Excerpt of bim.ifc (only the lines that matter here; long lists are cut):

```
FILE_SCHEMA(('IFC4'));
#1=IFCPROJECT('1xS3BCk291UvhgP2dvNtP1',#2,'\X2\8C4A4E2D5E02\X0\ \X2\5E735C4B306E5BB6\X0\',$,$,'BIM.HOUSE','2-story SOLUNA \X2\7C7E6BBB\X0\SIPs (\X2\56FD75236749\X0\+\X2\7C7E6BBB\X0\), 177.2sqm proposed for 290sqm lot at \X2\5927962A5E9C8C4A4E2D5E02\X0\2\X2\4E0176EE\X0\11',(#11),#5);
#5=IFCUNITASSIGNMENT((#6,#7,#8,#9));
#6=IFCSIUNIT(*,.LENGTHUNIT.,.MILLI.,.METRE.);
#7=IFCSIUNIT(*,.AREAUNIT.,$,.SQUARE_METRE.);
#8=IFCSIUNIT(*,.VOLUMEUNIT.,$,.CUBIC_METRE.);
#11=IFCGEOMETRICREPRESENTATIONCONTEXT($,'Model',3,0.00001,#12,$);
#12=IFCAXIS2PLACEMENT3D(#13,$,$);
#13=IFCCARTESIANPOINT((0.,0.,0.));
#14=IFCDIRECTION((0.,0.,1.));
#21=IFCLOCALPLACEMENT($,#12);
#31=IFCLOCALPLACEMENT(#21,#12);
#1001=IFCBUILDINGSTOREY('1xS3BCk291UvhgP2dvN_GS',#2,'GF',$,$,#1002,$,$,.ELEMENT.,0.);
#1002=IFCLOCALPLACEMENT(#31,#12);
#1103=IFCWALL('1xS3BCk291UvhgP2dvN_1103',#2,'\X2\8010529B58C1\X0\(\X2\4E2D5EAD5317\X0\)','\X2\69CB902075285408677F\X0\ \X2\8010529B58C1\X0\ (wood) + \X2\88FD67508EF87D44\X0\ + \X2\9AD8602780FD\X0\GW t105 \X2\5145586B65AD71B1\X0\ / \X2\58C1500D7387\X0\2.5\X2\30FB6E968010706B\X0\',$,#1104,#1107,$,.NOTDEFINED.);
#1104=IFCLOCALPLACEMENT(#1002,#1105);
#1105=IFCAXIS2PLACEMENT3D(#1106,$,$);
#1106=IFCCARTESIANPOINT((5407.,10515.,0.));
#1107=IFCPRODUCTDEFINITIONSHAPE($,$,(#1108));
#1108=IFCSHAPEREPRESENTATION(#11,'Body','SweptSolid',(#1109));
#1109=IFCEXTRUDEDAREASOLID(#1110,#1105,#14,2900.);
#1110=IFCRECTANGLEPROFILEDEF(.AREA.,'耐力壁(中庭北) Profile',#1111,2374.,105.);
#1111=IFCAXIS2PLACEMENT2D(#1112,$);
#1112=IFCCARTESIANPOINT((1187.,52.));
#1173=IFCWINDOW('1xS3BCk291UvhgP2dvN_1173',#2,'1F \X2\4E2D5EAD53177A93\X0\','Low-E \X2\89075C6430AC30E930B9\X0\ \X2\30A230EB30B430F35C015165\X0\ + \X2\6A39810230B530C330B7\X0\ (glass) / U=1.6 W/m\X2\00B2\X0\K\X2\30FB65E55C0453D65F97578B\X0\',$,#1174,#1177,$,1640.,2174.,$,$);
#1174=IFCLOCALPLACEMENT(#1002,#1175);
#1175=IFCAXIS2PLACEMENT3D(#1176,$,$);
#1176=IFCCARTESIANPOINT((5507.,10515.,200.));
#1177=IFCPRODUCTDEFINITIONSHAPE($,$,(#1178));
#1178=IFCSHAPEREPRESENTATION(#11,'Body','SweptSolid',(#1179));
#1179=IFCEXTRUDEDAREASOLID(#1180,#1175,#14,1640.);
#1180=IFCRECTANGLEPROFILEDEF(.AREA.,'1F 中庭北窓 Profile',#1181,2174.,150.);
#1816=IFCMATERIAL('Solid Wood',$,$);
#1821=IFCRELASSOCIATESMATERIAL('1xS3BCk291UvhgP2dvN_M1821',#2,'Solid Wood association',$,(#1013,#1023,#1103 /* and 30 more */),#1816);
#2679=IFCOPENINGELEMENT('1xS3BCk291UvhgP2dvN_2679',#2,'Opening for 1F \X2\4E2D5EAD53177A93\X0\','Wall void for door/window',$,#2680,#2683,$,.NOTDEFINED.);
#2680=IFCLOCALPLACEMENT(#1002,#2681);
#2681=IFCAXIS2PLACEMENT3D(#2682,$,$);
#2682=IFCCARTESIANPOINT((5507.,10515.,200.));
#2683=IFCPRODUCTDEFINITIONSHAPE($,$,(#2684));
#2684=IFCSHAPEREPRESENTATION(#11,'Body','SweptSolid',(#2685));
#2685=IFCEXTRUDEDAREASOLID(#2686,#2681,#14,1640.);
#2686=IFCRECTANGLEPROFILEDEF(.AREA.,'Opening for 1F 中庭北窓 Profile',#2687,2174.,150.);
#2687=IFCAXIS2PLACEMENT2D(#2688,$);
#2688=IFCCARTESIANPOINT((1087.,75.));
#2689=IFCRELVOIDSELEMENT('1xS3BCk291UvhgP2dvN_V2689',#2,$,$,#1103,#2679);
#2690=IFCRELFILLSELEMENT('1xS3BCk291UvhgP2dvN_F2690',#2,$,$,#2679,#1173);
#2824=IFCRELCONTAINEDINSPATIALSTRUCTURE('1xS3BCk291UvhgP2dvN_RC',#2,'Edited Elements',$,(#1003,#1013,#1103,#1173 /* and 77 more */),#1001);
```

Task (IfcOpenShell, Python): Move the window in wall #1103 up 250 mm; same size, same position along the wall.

```python
import numpy as np
import ifcopenshell
import ifcopenshell.api.geometry
import ifcopenshell.util.placement
import ifcopenshell.util.unit

model = ifcopenshell.open("bim.ifc")
unit_scale = ifcopenshell.util.unit.calculate_unit_scale(model)

window = model.by_id(1173)
opening = window.FillsVoids[0].RelatingOpeningElement
dz = 250.0

shift = np.array([0.0, 0.0, dz])
# The window is not placed relative to its opening, so move both.
for product in (opening, window):
    matrix = ifcopenshell.util.placement.get_local_placement(product.ObjectPlacement)
    matrix[:3, 3] += shift
    ifcopenshell.api.geometry.edit_object_placement(model, product=product, matrix=matrix, is_si=False)

print(f"moved by {dz * unit_scale:+.3f} m")

model.write("bim_updated.ifc")
```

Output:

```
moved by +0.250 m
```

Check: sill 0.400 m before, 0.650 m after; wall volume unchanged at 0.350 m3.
